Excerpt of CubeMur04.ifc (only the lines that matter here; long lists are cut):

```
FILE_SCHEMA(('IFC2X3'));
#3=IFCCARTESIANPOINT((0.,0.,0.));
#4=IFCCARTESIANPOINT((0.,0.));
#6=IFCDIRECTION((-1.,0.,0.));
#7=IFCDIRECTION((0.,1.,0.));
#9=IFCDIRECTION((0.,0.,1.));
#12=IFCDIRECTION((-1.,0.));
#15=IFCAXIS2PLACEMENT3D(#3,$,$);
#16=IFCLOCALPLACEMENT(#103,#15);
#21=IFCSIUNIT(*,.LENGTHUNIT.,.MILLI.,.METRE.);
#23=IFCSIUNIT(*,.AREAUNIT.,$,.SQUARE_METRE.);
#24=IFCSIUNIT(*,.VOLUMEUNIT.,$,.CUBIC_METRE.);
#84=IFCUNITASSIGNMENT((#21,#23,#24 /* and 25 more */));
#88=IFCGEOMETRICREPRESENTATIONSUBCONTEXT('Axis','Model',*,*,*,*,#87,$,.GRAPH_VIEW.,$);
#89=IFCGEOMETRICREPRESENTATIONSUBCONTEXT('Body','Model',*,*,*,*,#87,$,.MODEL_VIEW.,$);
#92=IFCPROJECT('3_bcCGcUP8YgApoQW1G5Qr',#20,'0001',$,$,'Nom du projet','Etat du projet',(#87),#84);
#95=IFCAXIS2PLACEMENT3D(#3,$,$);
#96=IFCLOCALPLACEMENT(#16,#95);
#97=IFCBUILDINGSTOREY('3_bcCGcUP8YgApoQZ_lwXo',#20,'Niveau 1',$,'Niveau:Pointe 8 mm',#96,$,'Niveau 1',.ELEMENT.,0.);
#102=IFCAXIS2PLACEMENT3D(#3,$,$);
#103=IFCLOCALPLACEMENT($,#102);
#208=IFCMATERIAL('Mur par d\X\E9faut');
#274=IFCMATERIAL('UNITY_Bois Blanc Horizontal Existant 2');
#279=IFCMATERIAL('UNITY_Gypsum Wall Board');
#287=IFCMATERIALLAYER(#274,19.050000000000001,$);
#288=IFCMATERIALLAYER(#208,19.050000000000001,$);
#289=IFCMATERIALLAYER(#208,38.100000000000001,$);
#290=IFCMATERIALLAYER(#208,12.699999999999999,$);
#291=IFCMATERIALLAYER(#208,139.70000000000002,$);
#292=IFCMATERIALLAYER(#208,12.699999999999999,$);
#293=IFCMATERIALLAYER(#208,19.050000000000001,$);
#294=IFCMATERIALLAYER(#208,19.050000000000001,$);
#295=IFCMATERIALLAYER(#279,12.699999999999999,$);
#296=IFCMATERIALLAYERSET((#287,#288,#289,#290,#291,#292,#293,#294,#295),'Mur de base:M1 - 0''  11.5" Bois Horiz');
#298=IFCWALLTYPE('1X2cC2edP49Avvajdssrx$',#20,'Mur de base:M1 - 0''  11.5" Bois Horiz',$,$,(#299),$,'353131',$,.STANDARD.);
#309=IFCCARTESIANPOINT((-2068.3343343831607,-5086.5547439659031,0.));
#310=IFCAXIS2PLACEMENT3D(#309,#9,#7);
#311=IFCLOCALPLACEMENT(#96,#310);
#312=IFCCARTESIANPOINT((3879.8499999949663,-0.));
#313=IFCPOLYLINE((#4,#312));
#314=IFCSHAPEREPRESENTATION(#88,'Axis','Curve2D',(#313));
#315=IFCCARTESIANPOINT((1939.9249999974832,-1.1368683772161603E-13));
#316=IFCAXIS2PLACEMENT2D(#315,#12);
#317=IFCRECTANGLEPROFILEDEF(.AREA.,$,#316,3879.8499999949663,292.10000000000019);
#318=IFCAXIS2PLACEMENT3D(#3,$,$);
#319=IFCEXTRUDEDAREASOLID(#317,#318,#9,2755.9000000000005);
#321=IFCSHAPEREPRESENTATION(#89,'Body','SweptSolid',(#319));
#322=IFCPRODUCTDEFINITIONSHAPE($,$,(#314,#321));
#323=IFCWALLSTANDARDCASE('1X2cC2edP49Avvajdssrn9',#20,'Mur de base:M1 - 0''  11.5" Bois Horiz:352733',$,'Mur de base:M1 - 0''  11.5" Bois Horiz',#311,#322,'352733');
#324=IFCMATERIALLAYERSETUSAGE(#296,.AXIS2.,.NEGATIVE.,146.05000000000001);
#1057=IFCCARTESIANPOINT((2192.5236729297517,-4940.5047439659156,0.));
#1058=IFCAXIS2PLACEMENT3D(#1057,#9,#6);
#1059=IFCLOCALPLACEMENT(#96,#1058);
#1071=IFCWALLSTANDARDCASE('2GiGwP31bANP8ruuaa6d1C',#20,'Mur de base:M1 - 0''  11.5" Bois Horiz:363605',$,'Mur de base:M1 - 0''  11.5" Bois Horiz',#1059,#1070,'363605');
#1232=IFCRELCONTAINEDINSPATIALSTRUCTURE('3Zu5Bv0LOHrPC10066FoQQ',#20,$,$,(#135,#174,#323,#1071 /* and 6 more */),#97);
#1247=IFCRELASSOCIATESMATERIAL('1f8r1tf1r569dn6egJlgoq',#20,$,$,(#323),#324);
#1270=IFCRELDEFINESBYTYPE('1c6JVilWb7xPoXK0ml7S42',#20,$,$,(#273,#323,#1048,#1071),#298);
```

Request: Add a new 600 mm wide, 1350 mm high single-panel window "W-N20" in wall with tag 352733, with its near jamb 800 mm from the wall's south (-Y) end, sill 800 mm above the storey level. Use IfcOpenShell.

```python
import numpy as np
import ifcopenshell
import ifcopenshell.api.feature
import ifcopenshell.api.geometry
import ifcopenshell.api.root
import ifcopenshell.api.spatial
import ifcopenshell.api.type
import ifcopenshell.geom
import ifcopenshell.util.element
import ifcopenshell.util.placement
import ifcopenshell.util.representation
import ifcopenshell.util.shape
import ifcopenshell.util.unit

model = ifcopenshell.open("CubeMur04.ifc")
unit_scale = ifcopenshell.util.unit.calculate_unit_scale(model)
settings = ifcopenshell.geom.settings()


def volume(element):
    """Net volume in cubic metres, openings subtracted."""
    shape = ifcopenshell.geom.create_shape(settings, element)
    return ifcopenshell.util.shape.get_volume(shape.geometry)


wall = model.by_guid("1X2cC2edP49Avvajdssrn9")
storey = ifcopenshell.util.element.get_container(wall, ifc_class="IfcBuildingStorey")
context = ifcopenshell.util.representation.get_context(model, "Model", "Body", "MODEL_VIEW")
before = volume(wall)

width, height, from_end, sill = 0.6, 1.35, 0.8, 0.8  # metres

# The wall runs along its own X axis, and the end named is its -X end.
wall_shape = ifcopenshell.geom.create_shape(settings, wall)
x, y, z = ifcopenshell.util.shape.get_vertices(wall_shape.geometry).T
start = x.min() + from_end
face, thickness = float(y.min()), float(y.max() - y.min())
wall_matrix = ifcopenshell.util.placement.get_local_placement(wall.ObjectPlacement)
level = ifcopenshell.util.placement.get_local_placement(storey.ObjectPlacement)[2, 3]


def in_wall(x, y):
    """Placement at x, y metres in the wall's axes, at sill height."""
    matrix = wall_matrix.copy()
    matrix[:, 3] = wall_matrix @ np.array([x / unit_scale, y / unit_scale, 0.0, 1.0])
    matrix[2, 3] = level + sill / unit_scale
    return matrix


# Opening: a box that overshoots both wall faces by 50 mm.
opening = ifcopenshell.api.root.create_entity(model, ifc_class="IfcOpeningElement")
box = ifcopenshell.api.geometry.add_wall_representation(
    model, context=context, length=width, height=height, thickness=thickness + 0.1
)
ifcopenshell.api.geometry.assign_representation(model, product=opening, representation=box)
ifcopenshell.api.geometry.edit_object_placement(model, product=opening, matrix=in_wall(start, face - 0.05), is_si=False)
ifcopenshell.api.feature.add_feature(model, feature=opening, element=wall)

window = ifcopenshell.api.root.create_entity(model, ifc_class="IfcWindow", name="W-N20")
window.OverallWidth, window.OverallHeight = width / unit_scale, height / unit_scale
body = ifcopenshell.api.geometry.add_window_representation(
    model,
    context=context,
    overall_width=window.OverallWidth,
    overall_height=window.OverallHeight,
    partition_type="SINGLE_PANEL",
)
ifcopenshell.api.geometry.assign_representation(model, product=window, representation=body)
ifcopenshell.api.spatial.assign_container(model, products=[window], relating_structure=storey)
fills = ifcopenshell.api.feature.add_filling(model, opening=opening, element=window)
fills.OwnerHistory = window.OwnerHistory  # required in IFC2X3

# IFC2X3 keeps the operation on the window style.
style = ifcopenshell.api.root.create_entity(model, ifc_class="IfcWindowStyle", name="W-N20")
style.OperationType, style.ConstructionType = "SINGLE_PANEL", "NOTDEFINED"
style.ParameterTakesPrecedence = style.Sizeable = False
ifcopenshell.api.type.assign_type(model, related_objects=[window], relating_type=style)

# Centre the window in the wall's thickness.
ifcopenshell.api.geometry.edit_object_placement(model, product=window, matrix=in_wall(start, face), is_si=False)
window_shape = ifcopenshell.geom.create_shape(settings, window)
depth = ifcopenshell.util.shape.get_vertices(window_shape.geometry)[:, 1]
offset = face + thickness / 2 - (depth.min() + depth.max()) / 2
ifcopenshell.api.geometry.edit_object_placement(model, product=window, matrix=in_wall(start, offset), is_si=False)

after = volume(wall)

print(f"wall volume {before:.3f} -> {after:.3f} m3")

model.write("CubeMur04_edited.ifc")
```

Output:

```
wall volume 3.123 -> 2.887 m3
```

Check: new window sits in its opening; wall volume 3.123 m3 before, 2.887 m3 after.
